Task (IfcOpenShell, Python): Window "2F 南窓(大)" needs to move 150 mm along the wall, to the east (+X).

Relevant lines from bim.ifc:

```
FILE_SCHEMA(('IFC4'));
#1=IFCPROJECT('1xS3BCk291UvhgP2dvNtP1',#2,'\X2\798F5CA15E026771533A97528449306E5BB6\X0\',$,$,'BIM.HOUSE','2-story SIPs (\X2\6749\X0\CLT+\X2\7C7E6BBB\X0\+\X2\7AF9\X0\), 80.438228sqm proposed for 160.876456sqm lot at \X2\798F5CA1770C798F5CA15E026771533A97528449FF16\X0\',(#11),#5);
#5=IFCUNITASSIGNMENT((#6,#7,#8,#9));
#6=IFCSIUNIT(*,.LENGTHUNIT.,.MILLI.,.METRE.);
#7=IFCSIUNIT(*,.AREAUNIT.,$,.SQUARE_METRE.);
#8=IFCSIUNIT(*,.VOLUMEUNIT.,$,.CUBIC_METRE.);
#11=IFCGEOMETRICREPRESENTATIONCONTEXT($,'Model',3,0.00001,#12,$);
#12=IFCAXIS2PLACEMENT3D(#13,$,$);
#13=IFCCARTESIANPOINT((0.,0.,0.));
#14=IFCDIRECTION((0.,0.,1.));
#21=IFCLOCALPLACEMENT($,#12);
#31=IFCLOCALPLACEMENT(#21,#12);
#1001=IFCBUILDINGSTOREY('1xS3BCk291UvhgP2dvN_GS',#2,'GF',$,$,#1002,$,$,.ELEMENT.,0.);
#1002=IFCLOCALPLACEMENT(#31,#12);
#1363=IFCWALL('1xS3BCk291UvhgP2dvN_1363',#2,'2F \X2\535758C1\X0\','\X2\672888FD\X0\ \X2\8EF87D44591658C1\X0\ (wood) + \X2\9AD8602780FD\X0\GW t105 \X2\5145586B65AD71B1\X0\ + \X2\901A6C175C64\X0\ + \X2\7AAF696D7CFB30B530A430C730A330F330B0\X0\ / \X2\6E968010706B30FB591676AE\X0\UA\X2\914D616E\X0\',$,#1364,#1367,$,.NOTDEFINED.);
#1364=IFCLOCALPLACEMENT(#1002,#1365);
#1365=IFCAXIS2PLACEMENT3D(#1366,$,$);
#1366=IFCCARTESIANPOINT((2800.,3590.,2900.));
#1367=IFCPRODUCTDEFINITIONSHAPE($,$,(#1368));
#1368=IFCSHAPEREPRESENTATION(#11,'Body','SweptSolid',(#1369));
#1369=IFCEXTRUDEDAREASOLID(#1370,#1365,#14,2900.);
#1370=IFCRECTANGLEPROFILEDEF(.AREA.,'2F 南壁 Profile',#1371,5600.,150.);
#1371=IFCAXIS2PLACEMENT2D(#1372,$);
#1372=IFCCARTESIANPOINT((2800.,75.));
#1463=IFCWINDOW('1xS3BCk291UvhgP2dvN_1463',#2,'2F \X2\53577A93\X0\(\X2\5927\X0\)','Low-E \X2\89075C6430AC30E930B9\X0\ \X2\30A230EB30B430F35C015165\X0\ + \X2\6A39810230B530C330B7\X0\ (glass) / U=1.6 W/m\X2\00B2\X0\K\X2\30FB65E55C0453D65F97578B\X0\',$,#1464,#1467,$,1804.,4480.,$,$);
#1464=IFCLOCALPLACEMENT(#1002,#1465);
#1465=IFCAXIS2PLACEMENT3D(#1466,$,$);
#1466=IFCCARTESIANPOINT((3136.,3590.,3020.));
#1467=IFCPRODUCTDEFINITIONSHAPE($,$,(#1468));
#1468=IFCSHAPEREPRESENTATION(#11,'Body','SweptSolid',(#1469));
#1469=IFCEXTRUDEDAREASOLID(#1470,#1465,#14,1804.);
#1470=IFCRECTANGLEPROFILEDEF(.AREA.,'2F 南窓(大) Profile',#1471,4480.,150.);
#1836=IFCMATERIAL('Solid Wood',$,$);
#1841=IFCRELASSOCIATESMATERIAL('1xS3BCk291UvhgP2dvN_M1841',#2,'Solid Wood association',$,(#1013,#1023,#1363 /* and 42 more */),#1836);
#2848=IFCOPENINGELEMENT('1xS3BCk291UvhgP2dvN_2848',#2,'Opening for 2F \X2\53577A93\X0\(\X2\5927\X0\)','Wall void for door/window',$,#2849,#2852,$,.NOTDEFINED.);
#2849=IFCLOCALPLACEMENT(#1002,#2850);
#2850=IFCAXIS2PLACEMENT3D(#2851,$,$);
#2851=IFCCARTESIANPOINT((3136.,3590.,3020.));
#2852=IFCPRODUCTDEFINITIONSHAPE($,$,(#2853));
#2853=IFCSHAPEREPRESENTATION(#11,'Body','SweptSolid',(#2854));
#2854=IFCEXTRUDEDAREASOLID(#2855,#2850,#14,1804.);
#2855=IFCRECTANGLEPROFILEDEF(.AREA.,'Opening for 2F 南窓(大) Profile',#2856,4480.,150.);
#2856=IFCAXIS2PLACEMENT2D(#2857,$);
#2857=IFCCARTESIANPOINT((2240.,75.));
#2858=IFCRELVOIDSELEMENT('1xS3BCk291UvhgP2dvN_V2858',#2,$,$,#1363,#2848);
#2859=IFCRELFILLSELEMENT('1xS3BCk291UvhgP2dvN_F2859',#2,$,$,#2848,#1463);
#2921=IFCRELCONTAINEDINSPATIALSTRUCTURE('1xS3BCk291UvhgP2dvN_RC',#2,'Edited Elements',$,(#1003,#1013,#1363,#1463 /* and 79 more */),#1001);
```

```python
import ifcopenshell
import ifcopenshell.api.geometry
import ifcopenshell.util.placement

model = ifcopenshell.open("bim.ifc")

window = model.by_guid("1xS3BCk291UvhgP2dvN_1463")
opening = window.FillsVoids[0].RelatingOpeningElement
wall = opening.VoidsElements[0].RelatingBuildingElement

wall_matrix = ifcopenshell.util.placement.get_local_placement(wall.ObjectPlacement)
shift = wall_matrix[:3, 0] * 150.0
before = ifcopenshell.util.placement.get_local_placement(window.ObjectPlacement)[:3, 3].copy()

# The window is not placed relative to its opening, so move both.
for product in (opening, window):
    matrix = ifcopenshell.util.placement.get_local_placement(product.ObjectPlacement)
    matrix[:3, 3] += shift
    ifcopenshell.api.geometry.edit_object_placement(model, product=product, matrix=matrix, is_si=False)

after = ifcopenshell.util.placement.get_local_placement(window.ObjectPlacement)[:3, 3]
print("window moved by", (after - before).round(3) + 0.0)

model.write("bim_updated.ifc")
```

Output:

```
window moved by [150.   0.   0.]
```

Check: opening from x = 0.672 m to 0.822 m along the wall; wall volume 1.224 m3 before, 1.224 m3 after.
